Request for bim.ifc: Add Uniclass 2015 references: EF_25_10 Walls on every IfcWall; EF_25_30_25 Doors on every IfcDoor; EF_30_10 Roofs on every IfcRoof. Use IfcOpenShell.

First a look at what the model holds.

```python
import ifcopenshell

model = ifcopenshell.open("bim.ifc")
print(model.schema)
print("classifications:", [c.Name for c in model.by_type("IfcClassification")])
for ifc_class in ("IfcDoor", "IfcRoof", "IfcStair", "IfcWall", "IfcWindow"):
    print(ifc_class, len(model.by_type(ifc_class)))
```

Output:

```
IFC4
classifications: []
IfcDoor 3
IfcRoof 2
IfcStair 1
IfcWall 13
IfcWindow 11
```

```python
import ifcopenshell
import ifcopenshell.api.classification

model = ifcopenshell.open("bim.ifc")

system = ifcopenshell.api.classification.add_classification(model, classification="Uniclass 2015")

codes = {
    "IfcWall": ("EF_25_10", "Walls"),
    "IfcDoor": ("EF_25_30_25", "Doors"),
    "IfcRoof": ("EF_30_10", "Roofs"),
}
for ifc_class, (code, name) in codes.items():
    products = model.by_type(ifc_class)
    ifcopenshell.api.classification.add_reference(
        model, products=products, classification=system, identification=code, name=name
    )
    print(code, len(products))

model.write("bim_updated.ifc")
```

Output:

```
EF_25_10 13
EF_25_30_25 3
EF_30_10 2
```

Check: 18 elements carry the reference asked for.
